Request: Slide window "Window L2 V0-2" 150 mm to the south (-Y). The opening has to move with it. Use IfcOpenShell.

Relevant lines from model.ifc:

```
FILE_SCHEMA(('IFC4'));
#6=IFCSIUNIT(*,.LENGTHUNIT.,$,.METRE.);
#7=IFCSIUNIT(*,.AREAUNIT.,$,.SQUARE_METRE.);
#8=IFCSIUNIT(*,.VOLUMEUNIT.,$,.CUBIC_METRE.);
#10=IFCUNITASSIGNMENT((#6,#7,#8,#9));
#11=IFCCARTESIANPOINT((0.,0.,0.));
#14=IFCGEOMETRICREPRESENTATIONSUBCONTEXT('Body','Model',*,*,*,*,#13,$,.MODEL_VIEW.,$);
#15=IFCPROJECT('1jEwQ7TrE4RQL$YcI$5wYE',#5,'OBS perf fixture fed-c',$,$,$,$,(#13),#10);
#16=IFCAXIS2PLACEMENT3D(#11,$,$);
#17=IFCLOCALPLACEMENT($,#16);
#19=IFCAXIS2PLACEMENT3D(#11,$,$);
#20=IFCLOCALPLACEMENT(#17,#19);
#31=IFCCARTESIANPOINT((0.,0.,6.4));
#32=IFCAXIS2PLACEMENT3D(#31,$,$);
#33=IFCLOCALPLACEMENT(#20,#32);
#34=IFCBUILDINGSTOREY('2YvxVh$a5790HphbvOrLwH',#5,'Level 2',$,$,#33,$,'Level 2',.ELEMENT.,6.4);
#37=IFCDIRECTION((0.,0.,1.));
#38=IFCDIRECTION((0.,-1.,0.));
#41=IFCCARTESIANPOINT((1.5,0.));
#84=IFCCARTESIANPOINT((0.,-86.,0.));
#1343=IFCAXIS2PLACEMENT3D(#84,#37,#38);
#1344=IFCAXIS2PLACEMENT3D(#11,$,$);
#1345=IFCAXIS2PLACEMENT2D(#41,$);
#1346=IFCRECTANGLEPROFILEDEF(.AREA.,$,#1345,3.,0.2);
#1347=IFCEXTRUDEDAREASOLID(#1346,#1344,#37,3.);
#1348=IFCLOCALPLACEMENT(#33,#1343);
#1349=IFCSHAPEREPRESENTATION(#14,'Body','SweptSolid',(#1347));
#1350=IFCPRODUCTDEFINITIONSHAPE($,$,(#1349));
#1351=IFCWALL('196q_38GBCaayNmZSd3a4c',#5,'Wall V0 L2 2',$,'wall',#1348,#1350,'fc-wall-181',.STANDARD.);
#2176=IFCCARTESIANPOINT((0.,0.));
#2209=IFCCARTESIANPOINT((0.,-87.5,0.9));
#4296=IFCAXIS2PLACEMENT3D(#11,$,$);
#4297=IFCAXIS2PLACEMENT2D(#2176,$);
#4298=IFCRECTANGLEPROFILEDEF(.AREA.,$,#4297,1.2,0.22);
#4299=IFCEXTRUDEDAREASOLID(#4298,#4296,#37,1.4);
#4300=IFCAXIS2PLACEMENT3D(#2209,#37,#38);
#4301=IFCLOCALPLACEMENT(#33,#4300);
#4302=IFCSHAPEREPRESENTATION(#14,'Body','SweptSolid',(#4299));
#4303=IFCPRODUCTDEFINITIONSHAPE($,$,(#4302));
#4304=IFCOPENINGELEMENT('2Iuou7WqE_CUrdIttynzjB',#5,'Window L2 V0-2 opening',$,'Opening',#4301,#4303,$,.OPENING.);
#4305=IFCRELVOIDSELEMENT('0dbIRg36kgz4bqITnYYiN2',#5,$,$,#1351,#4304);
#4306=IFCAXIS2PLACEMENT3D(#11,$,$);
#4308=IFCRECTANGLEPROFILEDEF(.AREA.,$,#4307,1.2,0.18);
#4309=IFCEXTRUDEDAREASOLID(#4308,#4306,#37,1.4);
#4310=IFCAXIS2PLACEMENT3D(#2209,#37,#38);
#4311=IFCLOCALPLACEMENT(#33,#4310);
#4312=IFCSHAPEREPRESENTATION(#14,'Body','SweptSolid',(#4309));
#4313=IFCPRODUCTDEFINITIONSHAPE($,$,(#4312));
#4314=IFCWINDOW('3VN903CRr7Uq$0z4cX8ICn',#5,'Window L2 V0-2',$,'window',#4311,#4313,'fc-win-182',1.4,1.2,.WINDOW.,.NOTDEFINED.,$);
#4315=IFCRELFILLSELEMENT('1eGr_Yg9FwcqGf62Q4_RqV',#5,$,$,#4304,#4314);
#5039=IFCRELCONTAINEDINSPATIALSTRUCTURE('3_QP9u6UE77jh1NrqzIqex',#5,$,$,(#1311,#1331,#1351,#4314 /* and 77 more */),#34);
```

```python
import ifcopenshell
import ifcopenshell.api.geometry
import ifcopenshell.util.placement
import ifcopenshell.util.unit

model = ifcopenshell.open("model.ifc")
unit_scale = ifcopenshell.util.unit.calculate_unit_scale(model)

window = model.by_id(4314)
opening = window.FillsVoids[0].RelatingOpeningElement
wall = opening.VoidsElements[0].RelatingBuildingElement

wall_matrix = ifcopenshell.util.placement.get_local_placement(wall.ObjectPlacement)
shift = wall_matrix[:3, 0] * 0.15 / unit_scale
before = ifcopenshell.util.placement.get_local_placement(window.ObjectPlacement)[:3, 3].copy()

# The window is not placed relative to its opening, so move both.
for product in (opening, window):
    matrix = ifcopenshell.util.placement.get_local_placement(product.ObjectPlacement)
    matrix[:3, 3] += shift
    ifcopenshell.api.geometry.edit_object_placement(model, product=product, matrix=matrix, is_si=False)

after = ifcopenshell.util.placement.get_local_placement(window.ObjectPlacement)[:3, 3]
print("window moved by", (after - before).round(3) + 0.0)

model.write("model_updated.ifc")
```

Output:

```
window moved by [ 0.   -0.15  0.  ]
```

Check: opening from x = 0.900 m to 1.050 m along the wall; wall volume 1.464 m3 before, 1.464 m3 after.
